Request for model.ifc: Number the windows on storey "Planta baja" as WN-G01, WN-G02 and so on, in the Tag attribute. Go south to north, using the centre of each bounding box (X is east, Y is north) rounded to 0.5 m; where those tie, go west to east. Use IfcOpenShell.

First a look at what the model holds.

```python
import ifcopenshell
import ifcopenshell.util.element
import ifcopenshell.util.placement

model = ifcopenshell.open("model.ifc")
print(model.schema)
storey = next(s for s in model.by_type("IfcBuildingStorey") if s.Name == "Planta baja")
windows = [e for e in ifcopenshell.util.element.get_decomposition(storey) if e.is_a("IfcWindow")]
for e in sorted(windows, key=lambda e: e.id()):
    origin = ifcopenshell.util.placement.get_local_placement(e.ObjectPlacement)[:3, 3]
    print(e.id(), e.Tag, e.Name, origin.round(2) + 0.0, sep=" | ")
```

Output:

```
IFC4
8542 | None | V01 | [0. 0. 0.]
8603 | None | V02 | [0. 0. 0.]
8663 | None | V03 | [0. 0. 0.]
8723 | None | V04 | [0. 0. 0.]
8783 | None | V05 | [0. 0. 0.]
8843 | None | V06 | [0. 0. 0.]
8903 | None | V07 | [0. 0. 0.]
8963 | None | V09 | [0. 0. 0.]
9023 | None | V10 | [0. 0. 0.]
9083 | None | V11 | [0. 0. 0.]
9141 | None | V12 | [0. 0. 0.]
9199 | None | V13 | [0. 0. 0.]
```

```python
import ifcopenshell
import ifcopenshell.geom
import ifcopenshell.util.element
import ifcopenshell.util.shape

model = ifcopenshell.open("model.ifc")
settings = ifcopenshell.geom.settings()
settings.set("use-world-coords", True)


def centre(element):
    shape = ifcopenshell.geom.create_shape(settings, element)
    return ifcopenshell.util.shape.get_bbox_centroid(shape.geometry)


storey = next(s for s in model.by_type("IfcBuildingStorey") if s.Name == "Planta baja")
windows = [e for e in ifcopenshell.util.element.get_decomposition(storey) if e.is_a("IfcWindow")]

# Insertion points can sit at a corner or the storey origin, so sort by the geometry (in metres).
centres = {e: centre(e) for e in windows}
windows.sort(key=lambda e: (round(centres[e][1] / 0.5), centres[e][0]))

for i, e in enumerate(windows, start=1):
    number = f"WN-G{i:02d}"
    e.Tag = number
    print(e.id(), number)

model.write("model_updated.ifc")
```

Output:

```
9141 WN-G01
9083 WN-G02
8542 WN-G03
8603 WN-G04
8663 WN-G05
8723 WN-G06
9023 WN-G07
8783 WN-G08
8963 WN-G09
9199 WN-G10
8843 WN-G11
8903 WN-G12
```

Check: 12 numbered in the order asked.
